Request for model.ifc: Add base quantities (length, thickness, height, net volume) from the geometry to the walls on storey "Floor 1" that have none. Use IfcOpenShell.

First a look at what the model holds.

```python
import ifcopenshell
import ifcopenshell.util.element
import ifcopenshell.util.unit

model = ifcopenshell.open("model.ifc")
print(model.schema)
for unit_type in ("LENGTHUNIT", "AREAUNIT", "VOLUMEUNIT"):
    print(unit_type, ifcopenshell.util.unit.calculate_unit_scale(model, unit_type))
storey = next(s for s in model.by_type("IfcBuildingStorey") if s.Name == "Floor 1")
walls = [e for e in ifcopenshell.util.element.get_decomposition(storey) if e.is_a("IfcWall")]
for e in sorted(walls, key=lambda e: e.id()):
    print(e.id(), e.is_a(), e.Name, list(ifcopenshell.util.element.get_psets(e, qtos_only=True)), sep=" | ")
```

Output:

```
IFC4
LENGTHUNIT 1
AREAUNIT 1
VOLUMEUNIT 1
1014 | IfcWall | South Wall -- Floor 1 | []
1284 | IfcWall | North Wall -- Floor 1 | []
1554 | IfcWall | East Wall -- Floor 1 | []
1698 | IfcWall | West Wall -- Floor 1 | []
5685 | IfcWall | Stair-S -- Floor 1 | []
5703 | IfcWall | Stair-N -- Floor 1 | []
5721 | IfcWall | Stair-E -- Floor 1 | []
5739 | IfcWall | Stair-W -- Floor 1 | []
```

```python
import ifcopenshell
import ifcopenshell.api.pset
import ifcopenshell.geom
import ifcopenshell.util.element
import ifcopenshell.util.shape
import ifcopenshell.util.unit

model = ifcopenshell.open("model.ifc")
unit_scale = ifcopenshell.util.unit.calculate_unit_scale(model)
volume_scale = ifcopenshell.util.unit.calculate_unit_scale(model, "VOLUMEUNIT")
settings = ifcopenshell.geom.settings()

storey = next(s for s in model.by_type("IfcBuildingStorey") if s.Name == "Floor 1")
walls = [e for e in ifcopenshell.util.element.get_decomposition(storey) if e.is_a("IfcWall")]

for e in sorted(walls, key=lambda e: e.id()):
    if ifcopenshell.util.element.get_psets(e, qtos_only=True, should_inherit=False):
        continue
    # Geometry comes back in metres, in the element's own axes.
    shape = ifcopenshell.geom.create_shape(settings, e)
    values = {
        "Length": ifcopenshell.util.shape.get_x(shape.geometry) / unit_scale,
        "Width": ifcopenshell.util.shape.get_y(shape.geometry) / unit_scale,
        "Height": ifcopenshell.util.shape.get_z(shape.geometry) / unit_scale,
        "NetVolume": ifcopenshell.util.shape.get_volume(shape.geometry) / volume_scale,
    }
    qto = ifcopenshell.api.pset.add_qto(model, product=e, name="Qto_WallBaseQuantities")
    ifcopenshell.api.pset.edit_qto(model, qto=qto, properties=values)
    print(e.id(), {k: round(v, 3) for k, v in values.items()})

model.write("model_edited.ifc")
```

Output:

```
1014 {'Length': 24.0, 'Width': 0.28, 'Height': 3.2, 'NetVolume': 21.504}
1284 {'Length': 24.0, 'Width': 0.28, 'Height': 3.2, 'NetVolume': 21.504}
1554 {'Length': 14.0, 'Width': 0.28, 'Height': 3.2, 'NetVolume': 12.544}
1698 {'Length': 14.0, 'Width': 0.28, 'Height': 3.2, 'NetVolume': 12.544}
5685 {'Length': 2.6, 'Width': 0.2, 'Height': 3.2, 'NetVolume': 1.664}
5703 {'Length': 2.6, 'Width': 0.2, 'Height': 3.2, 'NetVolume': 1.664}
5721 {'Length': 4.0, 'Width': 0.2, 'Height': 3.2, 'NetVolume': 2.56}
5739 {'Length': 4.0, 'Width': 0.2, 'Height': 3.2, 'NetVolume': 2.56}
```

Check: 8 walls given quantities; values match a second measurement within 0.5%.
